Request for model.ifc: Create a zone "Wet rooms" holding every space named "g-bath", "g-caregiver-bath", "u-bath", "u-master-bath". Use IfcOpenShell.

First a look at what the model holds.

```python
import ifcopenshell

model = ifcopenshell.open("model.ifc")
print(model.schema)
seen = {}
for space in model.by_type("IfcSpace"):
    seen[space.LongName] = seen.get(space.LongName, 0) + 1
for name, count in sorted(seen.items(), key=str):
    print(count, "x", name)
print("zones:", [z.Name for z in model.by_type("IfcZone")][:20])
```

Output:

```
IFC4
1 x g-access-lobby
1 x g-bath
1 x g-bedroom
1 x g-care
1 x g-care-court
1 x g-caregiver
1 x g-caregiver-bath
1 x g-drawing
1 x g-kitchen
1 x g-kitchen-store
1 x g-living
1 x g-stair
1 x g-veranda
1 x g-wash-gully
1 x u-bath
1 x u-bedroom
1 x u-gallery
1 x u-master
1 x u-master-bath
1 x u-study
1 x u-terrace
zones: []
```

```python
import ifcopenshell
import ifcopenshell.api.group
import ifcopenshell.api.root

model = ifcopenshell.open("model.ifc")

names = {"g-bath", "g-caregiver-bath", "u-bath", "u-master-bath"}
spaces = [s for s in model.by_type("IfcSpace") if s.LongName in names]

zone = ifcopenshell.api.root.create_entity(model, ifc_class="IfcZone", name="Wet rooms")
ifcopenshell.api.group.assign_group(model, products=spaces, group=zone)
print(len(spaces), "spaces in", zone.Name)

model.write("model_updated.ifc")
```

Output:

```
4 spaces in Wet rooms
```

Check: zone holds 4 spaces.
